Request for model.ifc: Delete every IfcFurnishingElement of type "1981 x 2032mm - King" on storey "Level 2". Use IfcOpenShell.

First a look at what the model holds.

```python
import ifcopenshell
import ifcopenshell.util.element

model = ifcopenshell.open("model.ifc")
print(model.schema)
storey = next(s for s in model.by_type("IfcBuildingStorey") if s.Name == "Level 2")
furniture = [e for e in ifcopenshell.util.element.get_decomposition(storey) if e.is_a("IfcFurnishingElement")]
seen = {}
for e in furniture:
    element_type = ifcopenshell.util.element.get_type(e)
    name = element_type.Name if element_type not in (None, e) else None
    seen[name] = seen.get(name, 0) + 1
for name, count in sorted(seen.items(), key=str):
    print(count, "x", name)
```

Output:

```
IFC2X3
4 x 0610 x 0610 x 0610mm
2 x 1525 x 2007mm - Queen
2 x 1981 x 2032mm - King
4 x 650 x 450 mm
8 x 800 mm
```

```python
import ifcopenshell
import ifcopenshell.api.root
import ifcopenshell.util.element

model = ifcopenshell.open("model.ifc")

storey = next(s for s in model.by_type("IfcBuildingStorey") if s.Name == "Level 2")
furniture = [e for e in ifcopenshell.util.element.get_decomposition(storey) if e.is_a("IfcFurnishingElement")]
targets = [e for e in furniture if (t := ifcopenshell.util.element.get_type(e)) not in (None, e) and t.Name == "1981 x 2032mm - King"]

for e in targets:
    ifcopenshell.api.root.remove_product(model, product=e)
print(len(targets), "removed")

model.write("model_edited.ifc")
```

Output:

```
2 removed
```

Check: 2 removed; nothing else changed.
